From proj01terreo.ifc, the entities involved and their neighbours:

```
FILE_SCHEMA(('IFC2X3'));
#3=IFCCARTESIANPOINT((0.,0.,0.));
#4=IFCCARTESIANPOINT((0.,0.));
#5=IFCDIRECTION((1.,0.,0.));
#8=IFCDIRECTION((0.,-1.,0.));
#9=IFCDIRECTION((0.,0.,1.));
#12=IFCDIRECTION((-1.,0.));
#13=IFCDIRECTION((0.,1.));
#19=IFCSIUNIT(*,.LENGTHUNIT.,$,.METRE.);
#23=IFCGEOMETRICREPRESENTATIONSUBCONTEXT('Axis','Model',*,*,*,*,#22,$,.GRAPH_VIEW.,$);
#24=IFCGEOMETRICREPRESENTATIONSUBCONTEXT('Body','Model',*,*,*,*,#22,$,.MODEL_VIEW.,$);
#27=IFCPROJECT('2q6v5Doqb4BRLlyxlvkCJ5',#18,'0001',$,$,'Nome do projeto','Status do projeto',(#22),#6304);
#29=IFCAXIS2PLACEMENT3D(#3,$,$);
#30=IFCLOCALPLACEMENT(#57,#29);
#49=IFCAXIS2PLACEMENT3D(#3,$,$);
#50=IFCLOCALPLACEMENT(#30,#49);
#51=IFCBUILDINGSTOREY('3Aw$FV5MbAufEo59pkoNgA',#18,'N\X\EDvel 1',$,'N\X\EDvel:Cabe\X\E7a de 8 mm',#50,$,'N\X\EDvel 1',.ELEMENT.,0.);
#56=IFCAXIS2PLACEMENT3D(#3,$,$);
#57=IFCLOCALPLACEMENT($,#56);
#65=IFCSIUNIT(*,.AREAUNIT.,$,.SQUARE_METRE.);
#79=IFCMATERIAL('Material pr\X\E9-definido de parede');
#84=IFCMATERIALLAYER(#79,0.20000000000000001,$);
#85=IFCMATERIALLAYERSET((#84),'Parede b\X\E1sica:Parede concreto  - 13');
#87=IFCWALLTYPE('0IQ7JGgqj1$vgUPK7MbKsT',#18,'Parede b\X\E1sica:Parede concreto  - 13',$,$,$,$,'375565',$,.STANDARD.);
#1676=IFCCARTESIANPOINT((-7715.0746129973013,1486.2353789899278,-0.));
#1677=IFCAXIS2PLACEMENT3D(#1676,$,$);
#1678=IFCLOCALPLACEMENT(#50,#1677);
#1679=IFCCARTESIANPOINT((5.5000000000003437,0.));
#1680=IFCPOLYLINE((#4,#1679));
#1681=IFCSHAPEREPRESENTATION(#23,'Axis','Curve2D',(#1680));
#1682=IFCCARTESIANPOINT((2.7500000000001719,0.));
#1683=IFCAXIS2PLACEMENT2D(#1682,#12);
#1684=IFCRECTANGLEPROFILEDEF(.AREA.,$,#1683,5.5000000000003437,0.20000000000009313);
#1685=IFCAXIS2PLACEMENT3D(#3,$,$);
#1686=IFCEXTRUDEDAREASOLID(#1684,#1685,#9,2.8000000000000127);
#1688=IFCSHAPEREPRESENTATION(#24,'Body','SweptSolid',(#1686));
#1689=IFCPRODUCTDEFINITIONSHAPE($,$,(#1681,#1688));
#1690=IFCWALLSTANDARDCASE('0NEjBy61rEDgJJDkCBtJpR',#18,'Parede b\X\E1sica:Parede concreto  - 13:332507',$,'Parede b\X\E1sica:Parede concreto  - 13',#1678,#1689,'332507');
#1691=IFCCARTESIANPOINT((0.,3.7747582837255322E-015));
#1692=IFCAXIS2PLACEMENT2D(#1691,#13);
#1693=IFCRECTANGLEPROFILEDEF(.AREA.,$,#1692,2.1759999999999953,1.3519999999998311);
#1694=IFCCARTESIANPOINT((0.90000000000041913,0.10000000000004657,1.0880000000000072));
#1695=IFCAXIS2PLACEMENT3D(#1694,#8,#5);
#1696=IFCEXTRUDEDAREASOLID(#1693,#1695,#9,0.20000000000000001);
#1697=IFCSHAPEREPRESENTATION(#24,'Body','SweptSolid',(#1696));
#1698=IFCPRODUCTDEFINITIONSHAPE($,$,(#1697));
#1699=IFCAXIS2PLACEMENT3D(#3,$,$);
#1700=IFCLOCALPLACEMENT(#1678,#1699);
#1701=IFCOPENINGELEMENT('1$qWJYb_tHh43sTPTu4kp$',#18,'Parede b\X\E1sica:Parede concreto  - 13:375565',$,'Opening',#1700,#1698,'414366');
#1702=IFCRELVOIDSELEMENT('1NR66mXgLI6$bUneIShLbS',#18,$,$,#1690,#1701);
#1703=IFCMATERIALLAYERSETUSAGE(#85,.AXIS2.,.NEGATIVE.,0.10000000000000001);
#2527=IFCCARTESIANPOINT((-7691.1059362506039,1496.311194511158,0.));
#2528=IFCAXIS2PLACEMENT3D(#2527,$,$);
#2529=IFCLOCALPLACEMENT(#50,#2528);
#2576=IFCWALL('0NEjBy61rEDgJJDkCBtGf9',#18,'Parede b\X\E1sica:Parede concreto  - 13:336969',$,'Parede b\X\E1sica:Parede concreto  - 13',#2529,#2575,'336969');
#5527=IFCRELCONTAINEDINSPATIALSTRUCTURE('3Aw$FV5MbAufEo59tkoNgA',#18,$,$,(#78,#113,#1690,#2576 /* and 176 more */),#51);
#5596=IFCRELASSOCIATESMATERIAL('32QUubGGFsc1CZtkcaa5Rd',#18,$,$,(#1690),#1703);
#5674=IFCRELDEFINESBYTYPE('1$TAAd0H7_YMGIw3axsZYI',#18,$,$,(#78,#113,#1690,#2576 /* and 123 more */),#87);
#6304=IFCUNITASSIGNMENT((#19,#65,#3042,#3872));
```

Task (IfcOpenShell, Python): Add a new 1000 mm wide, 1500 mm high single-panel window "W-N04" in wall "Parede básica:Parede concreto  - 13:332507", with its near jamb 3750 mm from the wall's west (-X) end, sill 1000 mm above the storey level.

```python
import numpy as np
import ifcopenshell
import ifcopenshell.api.feature
import ifcopenshell.api.geometry
import ifcopenshell.api.root
import ifcopenshell.api.spatial
import ifcopenshell.api.type
import ifcopenshell.geom
import ifcopenshell.util.element
import ifcopenshell.util.placement
import ifcopenshell.util.representation
import ifcopenshell.util.shape
import ifcopenshell.util.unit

model = ifcopenshell.open("proj01terreo.ifc")
unit_scale = ifcopenshell.util.unit.calculate_unit_scale(model)
settings = ifcopenshell.geom.settings()


def volume(element):
    """Net volume in cubic metres, openings subtracted."""
    shape = ifcopenshell.geom.create_shape(settings, element)
    return ifcopenshell.util.shape.get_volume(shape.geometry)


wall = model.by_id(1690)
storey = ifcopenshell.util.element.get_container(wall, ifc_class="IfcBuildingStorey")
context = ifcopenshell.util.representation.get_context(model, "Model", "Body", "MODEL_VIEW")
before = volume(wall)

width, height, from_end, sill = 1, 1.5, 3.75, 1  # metres

# The wall runs along its own X axis, and the end named is its -X end.
wall_shape = ifcopenshell.geom.create_shape(settings, wall)
x, y, z = ifcopenshell.util.shape.get_vertices(wall_shape.geometry).T
start = x.min() + from_end
face, thickness = float(y.min()), float(y.max() - y.min())
wall_matrix = ifcopenshell.util.placement.get_local_placement(wall.ObjectPlacement)
level = ifcopenshell.util.placement.get_local_placement(storey.ObjectPlacement)[2, 3]


def in_wall(x, y):
    """Placement at x, y metres in the wall's axes, at sill height."""
    matrix = wall_matrix.copy()
    matrix[:, 3] = wall_matrix @ np.array([x / unit_scale, y / unit_scale, 0.0, 1.0])
    matrix[2, 3] = level + sill / unit_scale
    return matrix


# Opening: a box that overshoots both wall faces by 50 mm.
opening = ifcopenshell.api.root.create_entity(model, ifc_class="IfcOpeningElement")
box = ifcopenshell.api.geometry.add_wall_representation(
    model, context=context, length=width, height=height, thickness=thickness + 0.1
)
ifcopenshell.api.geometry.assign_representation(model, product=opening, representation=box)
ifcopenshell.api.geometry.edit_object_placement(model, product=opening, matrix=in_wall(start, face - 0.05), is_si=False)
ifcopenshell.api.feature.add_feature(model, feature=opening, element=wall)

window = ifcopenshell.api.root.create_entity(model, ifc_class="IfcWindow", name="W-N04")
window.OverallWidth, window.OverallHeight = width / unit_scale, height / unit_scale
body = ifcopenshell.api.geometry.add_window_representation(
    model,
    context=context,
    overall_width=window.OverallWidth,
    overall_height=window.OverallHeight,
    partition_type="SINGLE_PANEL",
)
ifcopenshell.api.geometry.assign_representation(model, product=window, representation=body)
ifcopenshell.api.spatial.assign_container(model, products=[window], relating_structure=storey)
fills = ifcopenshell.api.feature.add_filling(model, opening=opening, element=window)
fills.OwnerHistory = window.OwnerHistory  # required in IFC2X3

# IFC2X3 keeps the operation on the window style.
style = ifcopenshell.api.root.create_entity(model, ifc_class="IfcWindowStyle", name="W-N04")
style.OperationType, style.ConstructionType = "SINGLE_PANEL", "NOTDEFINED"
style.ParameterTakesPrecedence = style.Sizeable = False
ifcopenshell.api.type.assign_type(model, related_objects=[window], relating_type=style)

# Centre the window in the wall's thickness.
ifcopenshell.api.geometry.edit_object_placement(model, product=window, matrix=in_wall(start, face), is_si=False)
window_shape = ifcopenshell.geom.create_shape(settings, window)
depth = ifcopenshell.util.shape.get_vertices(window_shape.geometry)[:, 1]
offset = face + thickness / 2 - (depth.min() + depth.max()) / 2
ifcopenshell.api.geometry.edit_object_placement(model, product=window, matrix=in_wall(start, offset), is_si=False)

after = volume(wall)

print(f"wall volume {before:.3f} -> {after:.3f} m3")

model.write("proj01terreo_rev.ifc")
```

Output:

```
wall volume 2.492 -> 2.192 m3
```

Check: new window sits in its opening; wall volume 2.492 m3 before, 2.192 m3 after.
